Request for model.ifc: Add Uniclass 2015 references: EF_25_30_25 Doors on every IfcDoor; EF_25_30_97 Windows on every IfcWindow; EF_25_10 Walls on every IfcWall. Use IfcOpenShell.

First a look at what the model holds.

```python
import ifcopenshell

model = ifcopenshell.open("model.ifc")
print(model.schema)
print("classifications:", [c.Name for c in model.by_type("IfcClassification")])
for ifc_class in ("IfcDoor", "IfcRoof", "IfcStair", "IfcWall", "IfcWindow"):
    print(ifc_class, len(model.by_type(ifc_class)))
```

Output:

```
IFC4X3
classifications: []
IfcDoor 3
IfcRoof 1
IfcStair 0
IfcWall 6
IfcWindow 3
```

```python
import ifcopenshell
import ifcopenshell.api.classification

model = ifcopenshell.open("model.ifc")

system = ifcopenshell.api.classification.add_classification(model, classification="Uniclass 2015")

codes = {
    "IfcDoor": ("EF_25_30_25", "Doors"),
    "IfcWindow": ("EF_25_30_97", "Windows"),
    "IfcWall": ("EF_25_10", "Walls"),
}
for ifc_class, (code, name) in codes.items():
    products = model.by_type(ifc_class)
    ifcopenshell.api.classification.add_reference(
        model, products=products, classification=system, identification=code, name=name
    )
    print(code, len(products))

model.write("model-out.ifc")
```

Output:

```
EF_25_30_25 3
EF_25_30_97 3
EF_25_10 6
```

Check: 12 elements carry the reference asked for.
